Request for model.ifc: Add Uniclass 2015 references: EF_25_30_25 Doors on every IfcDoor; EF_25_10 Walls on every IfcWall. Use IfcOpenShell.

First a look at what the model holds.

```python
import ifcopenshell

model = ifcopenshell.open("model.ifc")
print(model.schema)
print("classifications:", [c.Name for c in model.by_type("IfcClassification")])
for ifc_class in ("IfcDoor", "IfcRoof", "IfcStair", "IfcWall", "IfcWindow"):
    print(ifc_class, len(model.by_type(ifc_class)))
```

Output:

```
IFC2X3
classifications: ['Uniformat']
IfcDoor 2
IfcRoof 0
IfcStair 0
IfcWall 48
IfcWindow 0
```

```python
import ifcopenshell
import ifcopenshell.api.classification

model = ifcopenshell.open("model.ifc")

# IFC2X3 requires Source and Edition and has no link from the project to the system.
system = model.create_entity("IfcClassification", Source="NBS", Edition="2015", Name="Uniclass 2015")

codes = {
    "IfcDoor": ("EF_25_30_25", "Doors"),
    "IfcWall": ("EF_25_10", "Walls"),
}
for ifc_class, (code, name) in codes.items():
    products = model.by_type(ifc_class)
    ifcopenshell.api.classification.add_reference(
        model, products=products, classification=system, identification=code, name=name
    )
    print(code, len(products))

model.write("model_rev.ifc")
```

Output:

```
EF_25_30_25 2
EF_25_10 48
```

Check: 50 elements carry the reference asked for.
